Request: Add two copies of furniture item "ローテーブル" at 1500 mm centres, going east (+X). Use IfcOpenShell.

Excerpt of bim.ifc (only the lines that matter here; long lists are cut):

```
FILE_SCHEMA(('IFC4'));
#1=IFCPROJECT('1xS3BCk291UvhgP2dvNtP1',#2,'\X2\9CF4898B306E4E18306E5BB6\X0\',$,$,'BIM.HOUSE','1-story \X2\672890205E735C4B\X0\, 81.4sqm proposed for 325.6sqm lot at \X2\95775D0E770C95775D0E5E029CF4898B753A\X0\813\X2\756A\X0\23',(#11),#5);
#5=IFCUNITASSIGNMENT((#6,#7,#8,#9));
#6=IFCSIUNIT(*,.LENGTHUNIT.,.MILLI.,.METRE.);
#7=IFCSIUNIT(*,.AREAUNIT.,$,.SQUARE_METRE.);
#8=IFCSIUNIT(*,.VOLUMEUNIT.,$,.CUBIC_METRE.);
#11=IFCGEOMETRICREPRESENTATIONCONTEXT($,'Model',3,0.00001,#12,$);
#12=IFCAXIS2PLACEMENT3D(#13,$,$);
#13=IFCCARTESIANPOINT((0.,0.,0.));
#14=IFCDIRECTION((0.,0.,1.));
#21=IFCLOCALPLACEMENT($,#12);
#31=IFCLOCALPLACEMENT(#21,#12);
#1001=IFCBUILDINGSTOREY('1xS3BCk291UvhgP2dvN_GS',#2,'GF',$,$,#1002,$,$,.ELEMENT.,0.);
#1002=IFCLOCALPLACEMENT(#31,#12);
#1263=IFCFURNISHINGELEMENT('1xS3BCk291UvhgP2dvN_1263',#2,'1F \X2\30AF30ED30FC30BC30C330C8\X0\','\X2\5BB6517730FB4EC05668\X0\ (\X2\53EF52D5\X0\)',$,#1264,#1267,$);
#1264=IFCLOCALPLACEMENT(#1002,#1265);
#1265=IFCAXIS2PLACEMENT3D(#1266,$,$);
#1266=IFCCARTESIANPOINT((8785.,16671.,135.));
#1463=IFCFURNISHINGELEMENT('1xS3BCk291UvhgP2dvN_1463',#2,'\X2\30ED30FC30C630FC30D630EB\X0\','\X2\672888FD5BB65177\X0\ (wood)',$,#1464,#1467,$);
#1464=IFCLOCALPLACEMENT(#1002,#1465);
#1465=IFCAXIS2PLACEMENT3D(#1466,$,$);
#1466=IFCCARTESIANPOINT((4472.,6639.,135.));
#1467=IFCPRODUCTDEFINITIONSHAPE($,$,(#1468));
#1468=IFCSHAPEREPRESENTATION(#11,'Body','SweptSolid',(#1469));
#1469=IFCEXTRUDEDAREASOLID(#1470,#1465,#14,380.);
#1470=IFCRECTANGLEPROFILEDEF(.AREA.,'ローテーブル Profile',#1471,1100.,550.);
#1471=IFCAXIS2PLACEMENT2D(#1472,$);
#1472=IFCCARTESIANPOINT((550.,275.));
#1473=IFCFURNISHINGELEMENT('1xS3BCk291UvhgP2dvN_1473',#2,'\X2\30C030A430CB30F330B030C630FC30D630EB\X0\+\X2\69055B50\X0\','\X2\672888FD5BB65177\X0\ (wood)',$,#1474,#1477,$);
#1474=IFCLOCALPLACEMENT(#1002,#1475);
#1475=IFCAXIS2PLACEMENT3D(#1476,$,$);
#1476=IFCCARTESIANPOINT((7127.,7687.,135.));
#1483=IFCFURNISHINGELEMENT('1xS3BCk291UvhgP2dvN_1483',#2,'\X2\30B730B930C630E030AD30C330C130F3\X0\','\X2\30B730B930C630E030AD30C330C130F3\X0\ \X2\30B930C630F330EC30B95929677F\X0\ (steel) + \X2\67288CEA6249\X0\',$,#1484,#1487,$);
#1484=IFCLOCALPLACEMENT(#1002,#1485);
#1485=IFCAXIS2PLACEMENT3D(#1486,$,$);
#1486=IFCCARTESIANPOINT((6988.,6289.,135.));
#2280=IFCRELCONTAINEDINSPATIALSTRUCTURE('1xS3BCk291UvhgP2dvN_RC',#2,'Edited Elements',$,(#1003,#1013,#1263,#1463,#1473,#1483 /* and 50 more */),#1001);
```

```python
import numpy as np
import ifcopenshell
import ifcopenshell.api.geometry
import ifcopenshell.api.root
import ifcopenshell.util.element
import ifcopenshell.util.placement
import ifcopenshell.util.unit

model = ifcopenshell.open("bim.ifc")
unit_scale = ifcopenshell.util.unit.calculate_unit_scale(model)


def reuse_history(source, copy):
    """copy_class also copies each property set's owner history, people and application; keep the originals."""
    for rel in copy.IsDefinedBy:
        if rel.is_a("IfcRelDefinesByProperties") and (history := rel.RelatingPropertyDefinition.OwnerHistory):
            rel.RelatingPropertyDefinition.OwnerHistory = source.OwnerHistory
            ifcopenshell.util.element.remove_deep2(model, history)


source = model.by_guid("1xS3BCk291UvhgP2dvN_1463")
base = ifcopenshell.util.placement.get_local_placement(source.ObjectPlacement)
step = np.array([1.0, 0.0, 0.0]) * 1.5 / unit_scale

for i in range(1, 3):
    copy = ifcopenshell.api.root.copy_class(model, product=source)
    copy.Representation = ifcopenshell.util.element.copy_deep(
        model, source.Representation, exclude=["IfcGeometricRepresentationContext", "IfcRepresentationMap"]
    )
    reuse_history(source, copy)
    matrix = base.copy()
    matrix[:3, 3] += i * step
    print("added at", matrix[:3, 3].round(3) + 0.0)
    ifcopenshell.api.geometry.edit_object_placement(model, product=copy, matrix=matrix, is_si=False)

model.write("bim_rev.ifc")
```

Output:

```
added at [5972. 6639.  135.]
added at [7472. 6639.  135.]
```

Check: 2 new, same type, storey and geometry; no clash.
